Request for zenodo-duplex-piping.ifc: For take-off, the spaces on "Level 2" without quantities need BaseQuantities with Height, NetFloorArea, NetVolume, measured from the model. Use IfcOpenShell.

First a look at what the model holds.

```python
import ifcopenshell
import ifcopenshell.util.element
import ifcopenshell.util.unit

model = ifcopenshell.open("zenodo-duplex-piping.ifc")
print(model.schema)
for unit_type in ("LENGTHUNIT", "AREAUNIT", "VOLUMEUNIT"):
    print(unit_type, ifcopenshell.util.unit.calculate_unit_scale(model, unit_type))
storey = next(s for s in model.by_type("IfcBuildingStorey") if s.Name == "Level 2")
spaces = [e for e in ifcopenshell.util.element.get_decomposition(storey) if e.is_a("IfcSpace")]
for e in sorted(spaces, key=lambda e: e.id()):
    print(e.id(), e.is_a(), e.Name, list(ifcopenshell.util.element.get_psets(e, qtos_only=True)), sep=" | ")
```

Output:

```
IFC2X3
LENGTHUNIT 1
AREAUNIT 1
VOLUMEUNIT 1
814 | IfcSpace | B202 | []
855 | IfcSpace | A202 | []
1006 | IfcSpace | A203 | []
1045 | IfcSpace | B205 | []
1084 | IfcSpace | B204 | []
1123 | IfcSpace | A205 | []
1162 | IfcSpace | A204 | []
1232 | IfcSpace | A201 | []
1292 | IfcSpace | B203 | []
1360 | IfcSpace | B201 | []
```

```python
import ifcopenshell
import ifcopenshell.api.pset
import ifcopenshell.geom
import ifcopenshell.util.element
import ifcopenshell.util.shape
import ifcopenshell.util.unit

model = ifcopenshell.open("zenodo-duplex-piping.ifc")
unit_scale = ifcopenshell.util.unit.calculate_unit_scale(model)
area_scale = ifcopenshell.util.unit.calculate_unit_scale(model, "AREAUNIT")
volume_scale = ifcopenshell.util.unit.calculate_unit_scale(model, "VOLUMEUNIT")
settings = ifcopenshell.geom.settings()

storey = next(s for s in model.by_type("IfcBuildingStorey") if s.Name == "Level 2")
spaces = [e for e in ifcopenshell.util.element.get_decomposition(storey) if e.is_a("IfcSpace")]

for e in sorted(spaces, key=lambda e: e.id()):
    if ifcopenshell.util.element.get_psets(e, qtos_only=True, should_inherit=False):
        continue
    # Geometry comes back in metres, in the element's own axes.
    shape = ifcopenshell.geom.create_shape(settings, e)
    values = {
        "Height": ifcopenshell.util.shape.get_z(shape.geometry) / unit_scale,
        "NetFloorArea": ifcopenshell.util.shape.get_footprint_area(shape.geometry) / area_scale,
        "NetVolume": ifcopenshell.util.shape.get_volume(shape.geometry) / volume_scale,
    }
    qto = ifcopenshell.api.pset.add_qto(model, product=e, name="BaseQuantities")
    ifcopenshell.api.pset.edit_qto(model, qto=qto, properties=values)
    print(e.id(), {k: round(v, 3) for k, v in values.items()})

model.write("zenodo-duplex-piping_v2.ifc")
```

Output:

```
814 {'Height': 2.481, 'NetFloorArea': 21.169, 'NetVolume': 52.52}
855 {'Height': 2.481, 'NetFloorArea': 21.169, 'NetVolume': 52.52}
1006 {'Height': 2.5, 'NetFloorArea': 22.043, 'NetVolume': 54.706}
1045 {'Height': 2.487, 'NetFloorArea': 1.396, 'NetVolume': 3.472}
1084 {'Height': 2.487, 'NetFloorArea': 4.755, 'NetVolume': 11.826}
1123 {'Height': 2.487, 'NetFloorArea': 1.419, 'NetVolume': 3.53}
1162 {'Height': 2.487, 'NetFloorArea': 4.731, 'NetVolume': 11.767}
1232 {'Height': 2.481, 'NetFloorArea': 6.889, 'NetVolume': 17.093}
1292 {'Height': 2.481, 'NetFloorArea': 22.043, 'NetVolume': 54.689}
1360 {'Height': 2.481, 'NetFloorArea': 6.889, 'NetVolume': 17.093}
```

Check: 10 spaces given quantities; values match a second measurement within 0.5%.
